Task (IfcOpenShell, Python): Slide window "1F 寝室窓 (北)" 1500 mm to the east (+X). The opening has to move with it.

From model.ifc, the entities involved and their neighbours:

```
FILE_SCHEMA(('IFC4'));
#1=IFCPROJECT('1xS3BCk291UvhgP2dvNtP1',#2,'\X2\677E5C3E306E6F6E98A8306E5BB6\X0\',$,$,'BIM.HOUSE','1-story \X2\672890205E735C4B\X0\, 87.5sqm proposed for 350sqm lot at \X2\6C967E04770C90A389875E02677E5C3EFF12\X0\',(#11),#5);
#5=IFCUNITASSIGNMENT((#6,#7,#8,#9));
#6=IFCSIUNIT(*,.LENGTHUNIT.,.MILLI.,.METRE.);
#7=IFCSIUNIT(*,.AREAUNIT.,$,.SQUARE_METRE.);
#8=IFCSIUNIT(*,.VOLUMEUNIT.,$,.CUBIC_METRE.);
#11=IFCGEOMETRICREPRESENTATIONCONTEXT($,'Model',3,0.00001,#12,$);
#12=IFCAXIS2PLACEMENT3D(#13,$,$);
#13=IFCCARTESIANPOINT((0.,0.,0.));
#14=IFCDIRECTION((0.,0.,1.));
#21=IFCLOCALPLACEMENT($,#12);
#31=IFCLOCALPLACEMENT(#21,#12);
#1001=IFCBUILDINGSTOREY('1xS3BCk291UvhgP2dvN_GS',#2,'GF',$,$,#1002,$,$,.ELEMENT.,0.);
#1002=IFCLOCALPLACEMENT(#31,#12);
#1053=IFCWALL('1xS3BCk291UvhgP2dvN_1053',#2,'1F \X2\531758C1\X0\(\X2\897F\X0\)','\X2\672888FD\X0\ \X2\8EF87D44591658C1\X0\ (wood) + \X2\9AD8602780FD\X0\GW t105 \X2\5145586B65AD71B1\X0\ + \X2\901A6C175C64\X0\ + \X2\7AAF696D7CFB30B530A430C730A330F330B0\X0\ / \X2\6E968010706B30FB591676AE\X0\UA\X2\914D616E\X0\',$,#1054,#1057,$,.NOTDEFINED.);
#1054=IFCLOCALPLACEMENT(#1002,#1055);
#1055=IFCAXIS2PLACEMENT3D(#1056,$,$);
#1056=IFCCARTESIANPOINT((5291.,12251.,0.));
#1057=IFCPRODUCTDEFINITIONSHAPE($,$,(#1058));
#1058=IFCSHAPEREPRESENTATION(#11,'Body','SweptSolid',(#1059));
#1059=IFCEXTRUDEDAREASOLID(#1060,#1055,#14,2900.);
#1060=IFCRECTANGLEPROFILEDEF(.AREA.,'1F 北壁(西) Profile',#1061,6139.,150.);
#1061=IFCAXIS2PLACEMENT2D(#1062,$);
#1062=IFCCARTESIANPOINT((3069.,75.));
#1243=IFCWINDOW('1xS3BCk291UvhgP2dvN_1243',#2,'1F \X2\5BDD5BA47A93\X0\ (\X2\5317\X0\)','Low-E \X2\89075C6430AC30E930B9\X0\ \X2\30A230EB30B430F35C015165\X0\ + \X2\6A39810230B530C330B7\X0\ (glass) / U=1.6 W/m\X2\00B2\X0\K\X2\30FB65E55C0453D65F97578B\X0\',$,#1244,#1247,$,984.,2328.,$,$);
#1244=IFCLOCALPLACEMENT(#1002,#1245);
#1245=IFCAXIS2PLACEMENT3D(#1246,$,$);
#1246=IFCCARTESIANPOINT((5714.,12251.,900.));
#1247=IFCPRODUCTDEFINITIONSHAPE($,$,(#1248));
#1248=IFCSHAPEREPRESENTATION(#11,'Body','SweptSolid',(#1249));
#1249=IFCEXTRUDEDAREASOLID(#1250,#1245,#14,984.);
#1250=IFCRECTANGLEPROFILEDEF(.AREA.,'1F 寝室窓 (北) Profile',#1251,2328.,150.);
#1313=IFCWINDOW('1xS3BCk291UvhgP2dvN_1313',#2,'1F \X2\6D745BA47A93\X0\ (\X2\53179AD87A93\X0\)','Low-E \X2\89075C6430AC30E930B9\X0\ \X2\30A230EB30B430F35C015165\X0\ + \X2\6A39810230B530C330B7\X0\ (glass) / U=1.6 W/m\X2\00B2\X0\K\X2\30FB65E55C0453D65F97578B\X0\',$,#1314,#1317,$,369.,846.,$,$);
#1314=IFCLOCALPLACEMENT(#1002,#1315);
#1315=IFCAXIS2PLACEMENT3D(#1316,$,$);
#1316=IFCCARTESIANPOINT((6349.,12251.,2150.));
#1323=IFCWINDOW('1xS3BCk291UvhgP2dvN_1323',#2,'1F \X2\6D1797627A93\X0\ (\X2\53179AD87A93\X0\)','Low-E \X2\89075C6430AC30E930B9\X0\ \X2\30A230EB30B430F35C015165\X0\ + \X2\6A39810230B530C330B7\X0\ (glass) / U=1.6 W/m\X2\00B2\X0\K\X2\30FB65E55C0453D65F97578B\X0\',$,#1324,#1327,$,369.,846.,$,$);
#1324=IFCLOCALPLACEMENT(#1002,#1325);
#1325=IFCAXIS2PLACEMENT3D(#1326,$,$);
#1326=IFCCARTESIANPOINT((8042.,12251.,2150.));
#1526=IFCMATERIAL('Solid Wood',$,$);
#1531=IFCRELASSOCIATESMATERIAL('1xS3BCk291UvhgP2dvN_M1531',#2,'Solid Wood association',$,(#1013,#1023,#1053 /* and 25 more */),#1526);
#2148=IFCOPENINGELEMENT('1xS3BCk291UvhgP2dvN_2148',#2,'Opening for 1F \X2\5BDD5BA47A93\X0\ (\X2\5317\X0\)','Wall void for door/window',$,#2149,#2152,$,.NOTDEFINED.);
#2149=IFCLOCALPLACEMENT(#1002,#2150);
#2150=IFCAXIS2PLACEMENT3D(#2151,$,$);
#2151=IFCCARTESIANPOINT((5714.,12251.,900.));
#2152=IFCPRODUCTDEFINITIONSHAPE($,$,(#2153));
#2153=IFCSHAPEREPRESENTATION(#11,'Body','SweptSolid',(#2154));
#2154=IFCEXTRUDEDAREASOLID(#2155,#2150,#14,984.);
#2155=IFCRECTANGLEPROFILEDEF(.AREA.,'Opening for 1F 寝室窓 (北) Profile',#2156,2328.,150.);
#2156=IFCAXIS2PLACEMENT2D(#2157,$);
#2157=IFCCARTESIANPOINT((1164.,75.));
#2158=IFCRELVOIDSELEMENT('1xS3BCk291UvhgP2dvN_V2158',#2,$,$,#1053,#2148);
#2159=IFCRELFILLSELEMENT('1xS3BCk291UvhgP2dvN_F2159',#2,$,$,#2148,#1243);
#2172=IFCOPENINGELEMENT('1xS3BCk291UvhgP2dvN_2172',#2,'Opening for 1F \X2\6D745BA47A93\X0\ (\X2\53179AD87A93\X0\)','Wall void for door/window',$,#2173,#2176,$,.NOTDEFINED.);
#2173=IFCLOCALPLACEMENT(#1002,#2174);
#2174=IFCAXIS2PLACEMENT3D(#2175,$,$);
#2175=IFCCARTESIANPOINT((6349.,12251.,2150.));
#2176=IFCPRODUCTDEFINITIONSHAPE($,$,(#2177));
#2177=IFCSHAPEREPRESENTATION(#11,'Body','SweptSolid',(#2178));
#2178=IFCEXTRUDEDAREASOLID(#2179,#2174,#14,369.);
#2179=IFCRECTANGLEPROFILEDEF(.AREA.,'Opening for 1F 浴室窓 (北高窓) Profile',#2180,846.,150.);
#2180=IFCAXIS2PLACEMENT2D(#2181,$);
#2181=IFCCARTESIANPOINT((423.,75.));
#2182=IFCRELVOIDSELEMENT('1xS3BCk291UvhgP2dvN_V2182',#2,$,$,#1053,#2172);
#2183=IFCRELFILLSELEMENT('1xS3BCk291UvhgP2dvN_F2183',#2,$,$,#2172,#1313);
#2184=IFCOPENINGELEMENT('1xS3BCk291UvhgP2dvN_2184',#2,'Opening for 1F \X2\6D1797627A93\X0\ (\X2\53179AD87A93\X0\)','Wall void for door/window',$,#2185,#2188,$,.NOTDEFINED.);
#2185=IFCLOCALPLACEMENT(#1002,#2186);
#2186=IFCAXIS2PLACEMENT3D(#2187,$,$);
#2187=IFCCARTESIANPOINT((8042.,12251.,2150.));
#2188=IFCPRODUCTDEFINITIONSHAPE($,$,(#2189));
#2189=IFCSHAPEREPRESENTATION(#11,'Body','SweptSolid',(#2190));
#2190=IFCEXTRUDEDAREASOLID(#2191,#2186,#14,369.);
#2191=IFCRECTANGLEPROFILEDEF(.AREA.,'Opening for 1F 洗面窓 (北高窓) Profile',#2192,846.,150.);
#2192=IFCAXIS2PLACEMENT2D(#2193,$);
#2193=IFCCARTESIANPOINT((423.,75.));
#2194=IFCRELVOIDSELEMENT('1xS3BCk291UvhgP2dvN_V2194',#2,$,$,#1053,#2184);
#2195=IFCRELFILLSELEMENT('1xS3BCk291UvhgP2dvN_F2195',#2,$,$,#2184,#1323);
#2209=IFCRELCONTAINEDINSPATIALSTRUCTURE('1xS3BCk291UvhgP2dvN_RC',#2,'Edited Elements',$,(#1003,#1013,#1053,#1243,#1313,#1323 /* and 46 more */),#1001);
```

```python
import ifcopenshell
import ifcopenshell.api.geometry
import ifcopenshell.util.placement
import ifcopenshell.util.unit

model = ifcopenshell.open("model.ifc")
unit_scale = ifcopenshell.util.unit.calculate_unit_scale(model)

window = model.by_guid("1xS3BCk291UvhgP2dvN_1243")
opening = window.FillsVoids[0].RelatingOpeningElement
wall = opening.VoidsElements[0].RelatingBuildingElement

wall_matrix = ifcopenshell.util.placement.get_local_placement(wall.ObjectPlacement)
shift = wall_matrix[:3, 0] * 1.5 / unit_scale
before = ifcopenshell.util.placement.get_local_placement(window.ObjectPlacement)[:3, 3].copy()

# The window is not placed relative to its opening, so move both.
for product in (opening, window):
    matrix = ifcopenshell.util.placement.get_local_placement(product.ObjectPlacement)
    matrix[:3, 3] += shift
    ifcopenshell.api.geometry.edit_object_placement(model, product=product, matrix=matrix, is_si=False)

after = ifcopenshell.util.placement.get_local_placement(window.ObjectPlacement)[:3, 3]
print("window moved by", (after - before).round(3) + 0.0)

model.write("model-out.ifc")
```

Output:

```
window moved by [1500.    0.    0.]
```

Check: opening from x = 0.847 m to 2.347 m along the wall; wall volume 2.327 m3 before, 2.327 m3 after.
